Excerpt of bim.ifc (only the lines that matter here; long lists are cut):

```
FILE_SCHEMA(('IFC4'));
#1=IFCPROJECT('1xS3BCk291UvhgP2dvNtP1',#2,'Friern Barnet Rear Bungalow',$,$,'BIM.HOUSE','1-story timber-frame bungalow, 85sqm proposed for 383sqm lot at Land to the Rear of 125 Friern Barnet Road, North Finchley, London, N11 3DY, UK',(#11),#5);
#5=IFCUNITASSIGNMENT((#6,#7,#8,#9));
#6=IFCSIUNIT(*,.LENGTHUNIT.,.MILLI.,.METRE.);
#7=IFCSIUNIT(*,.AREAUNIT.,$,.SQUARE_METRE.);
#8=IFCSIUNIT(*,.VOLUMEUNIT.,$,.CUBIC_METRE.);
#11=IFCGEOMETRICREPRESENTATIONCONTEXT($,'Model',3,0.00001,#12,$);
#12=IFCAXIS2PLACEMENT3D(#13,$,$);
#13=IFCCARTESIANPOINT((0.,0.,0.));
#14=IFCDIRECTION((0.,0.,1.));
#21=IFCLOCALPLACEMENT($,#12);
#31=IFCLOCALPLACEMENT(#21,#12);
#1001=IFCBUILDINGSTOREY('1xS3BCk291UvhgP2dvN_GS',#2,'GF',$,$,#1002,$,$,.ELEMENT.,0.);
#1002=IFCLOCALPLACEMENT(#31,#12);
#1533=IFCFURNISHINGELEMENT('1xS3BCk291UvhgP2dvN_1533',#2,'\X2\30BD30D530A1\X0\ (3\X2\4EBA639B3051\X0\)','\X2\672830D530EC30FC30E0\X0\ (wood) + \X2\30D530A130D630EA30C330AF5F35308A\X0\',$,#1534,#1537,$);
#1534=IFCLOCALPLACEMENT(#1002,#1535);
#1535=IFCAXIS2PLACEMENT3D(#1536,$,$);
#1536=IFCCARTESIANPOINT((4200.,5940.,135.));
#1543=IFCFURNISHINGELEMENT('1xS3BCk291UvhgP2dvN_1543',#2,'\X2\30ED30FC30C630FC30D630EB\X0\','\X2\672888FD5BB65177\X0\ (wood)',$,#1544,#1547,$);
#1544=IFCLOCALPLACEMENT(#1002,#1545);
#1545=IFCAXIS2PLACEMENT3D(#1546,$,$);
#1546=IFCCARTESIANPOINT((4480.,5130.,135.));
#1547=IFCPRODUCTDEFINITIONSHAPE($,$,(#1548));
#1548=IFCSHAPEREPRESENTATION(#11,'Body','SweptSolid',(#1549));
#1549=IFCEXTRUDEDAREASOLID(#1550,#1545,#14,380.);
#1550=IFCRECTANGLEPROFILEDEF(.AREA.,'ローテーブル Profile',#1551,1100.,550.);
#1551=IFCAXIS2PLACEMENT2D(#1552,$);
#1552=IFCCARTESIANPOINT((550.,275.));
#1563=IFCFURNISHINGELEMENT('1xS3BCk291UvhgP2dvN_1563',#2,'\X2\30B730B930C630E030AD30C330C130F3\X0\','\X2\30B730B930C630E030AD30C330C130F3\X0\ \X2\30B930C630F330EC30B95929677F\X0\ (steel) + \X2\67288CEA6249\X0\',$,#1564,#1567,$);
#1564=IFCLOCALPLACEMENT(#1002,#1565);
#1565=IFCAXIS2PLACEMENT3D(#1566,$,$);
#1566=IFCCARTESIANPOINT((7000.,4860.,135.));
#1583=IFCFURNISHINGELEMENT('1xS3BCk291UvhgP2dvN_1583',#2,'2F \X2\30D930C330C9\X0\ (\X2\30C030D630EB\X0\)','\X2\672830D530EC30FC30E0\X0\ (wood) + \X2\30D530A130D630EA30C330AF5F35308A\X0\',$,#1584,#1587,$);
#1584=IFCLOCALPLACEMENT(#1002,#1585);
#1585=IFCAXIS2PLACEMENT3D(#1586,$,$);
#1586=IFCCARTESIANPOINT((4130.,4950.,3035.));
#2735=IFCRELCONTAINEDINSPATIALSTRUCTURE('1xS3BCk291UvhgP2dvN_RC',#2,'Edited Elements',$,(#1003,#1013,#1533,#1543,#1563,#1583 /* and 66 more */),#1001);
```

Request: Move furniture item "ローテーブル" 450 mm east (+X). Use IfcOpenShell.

```python
import ifcopenshell
import ifcopenshell.api.geometry
import ifcopenshell.util.placement
import ifcopenshell.util.unit

model = ifcopenshell.open("bim.ifc")
unit_scale = ifcopenshell.util.unit.calculate_unit_scale(model)

item = model.by_guid("1xS3BCk291UvhgP2dvN_1543")
matrix = ifcopenshell.util.placement.get_local_placement(item.ObjectPlacement)
matrix[0, 3] += 0.45 / unit_scale
ifcopenshell.api.geometry.edit_object_placement(model, product=item, matrix=matrix, is_si=False)

print(ifcopenshell.util.placement.get_local_placement(item.ObjectPlacement).round(3) + 0.0)

model.write("bim_rev.ifc")
```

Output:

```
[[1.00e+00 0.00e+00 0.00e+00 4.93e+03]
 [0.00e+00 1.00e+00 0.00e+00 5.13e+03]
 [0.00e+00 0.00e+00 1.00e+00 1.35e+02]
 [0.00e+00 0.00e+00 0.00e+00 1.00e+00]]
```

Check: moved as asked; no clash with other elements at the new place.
